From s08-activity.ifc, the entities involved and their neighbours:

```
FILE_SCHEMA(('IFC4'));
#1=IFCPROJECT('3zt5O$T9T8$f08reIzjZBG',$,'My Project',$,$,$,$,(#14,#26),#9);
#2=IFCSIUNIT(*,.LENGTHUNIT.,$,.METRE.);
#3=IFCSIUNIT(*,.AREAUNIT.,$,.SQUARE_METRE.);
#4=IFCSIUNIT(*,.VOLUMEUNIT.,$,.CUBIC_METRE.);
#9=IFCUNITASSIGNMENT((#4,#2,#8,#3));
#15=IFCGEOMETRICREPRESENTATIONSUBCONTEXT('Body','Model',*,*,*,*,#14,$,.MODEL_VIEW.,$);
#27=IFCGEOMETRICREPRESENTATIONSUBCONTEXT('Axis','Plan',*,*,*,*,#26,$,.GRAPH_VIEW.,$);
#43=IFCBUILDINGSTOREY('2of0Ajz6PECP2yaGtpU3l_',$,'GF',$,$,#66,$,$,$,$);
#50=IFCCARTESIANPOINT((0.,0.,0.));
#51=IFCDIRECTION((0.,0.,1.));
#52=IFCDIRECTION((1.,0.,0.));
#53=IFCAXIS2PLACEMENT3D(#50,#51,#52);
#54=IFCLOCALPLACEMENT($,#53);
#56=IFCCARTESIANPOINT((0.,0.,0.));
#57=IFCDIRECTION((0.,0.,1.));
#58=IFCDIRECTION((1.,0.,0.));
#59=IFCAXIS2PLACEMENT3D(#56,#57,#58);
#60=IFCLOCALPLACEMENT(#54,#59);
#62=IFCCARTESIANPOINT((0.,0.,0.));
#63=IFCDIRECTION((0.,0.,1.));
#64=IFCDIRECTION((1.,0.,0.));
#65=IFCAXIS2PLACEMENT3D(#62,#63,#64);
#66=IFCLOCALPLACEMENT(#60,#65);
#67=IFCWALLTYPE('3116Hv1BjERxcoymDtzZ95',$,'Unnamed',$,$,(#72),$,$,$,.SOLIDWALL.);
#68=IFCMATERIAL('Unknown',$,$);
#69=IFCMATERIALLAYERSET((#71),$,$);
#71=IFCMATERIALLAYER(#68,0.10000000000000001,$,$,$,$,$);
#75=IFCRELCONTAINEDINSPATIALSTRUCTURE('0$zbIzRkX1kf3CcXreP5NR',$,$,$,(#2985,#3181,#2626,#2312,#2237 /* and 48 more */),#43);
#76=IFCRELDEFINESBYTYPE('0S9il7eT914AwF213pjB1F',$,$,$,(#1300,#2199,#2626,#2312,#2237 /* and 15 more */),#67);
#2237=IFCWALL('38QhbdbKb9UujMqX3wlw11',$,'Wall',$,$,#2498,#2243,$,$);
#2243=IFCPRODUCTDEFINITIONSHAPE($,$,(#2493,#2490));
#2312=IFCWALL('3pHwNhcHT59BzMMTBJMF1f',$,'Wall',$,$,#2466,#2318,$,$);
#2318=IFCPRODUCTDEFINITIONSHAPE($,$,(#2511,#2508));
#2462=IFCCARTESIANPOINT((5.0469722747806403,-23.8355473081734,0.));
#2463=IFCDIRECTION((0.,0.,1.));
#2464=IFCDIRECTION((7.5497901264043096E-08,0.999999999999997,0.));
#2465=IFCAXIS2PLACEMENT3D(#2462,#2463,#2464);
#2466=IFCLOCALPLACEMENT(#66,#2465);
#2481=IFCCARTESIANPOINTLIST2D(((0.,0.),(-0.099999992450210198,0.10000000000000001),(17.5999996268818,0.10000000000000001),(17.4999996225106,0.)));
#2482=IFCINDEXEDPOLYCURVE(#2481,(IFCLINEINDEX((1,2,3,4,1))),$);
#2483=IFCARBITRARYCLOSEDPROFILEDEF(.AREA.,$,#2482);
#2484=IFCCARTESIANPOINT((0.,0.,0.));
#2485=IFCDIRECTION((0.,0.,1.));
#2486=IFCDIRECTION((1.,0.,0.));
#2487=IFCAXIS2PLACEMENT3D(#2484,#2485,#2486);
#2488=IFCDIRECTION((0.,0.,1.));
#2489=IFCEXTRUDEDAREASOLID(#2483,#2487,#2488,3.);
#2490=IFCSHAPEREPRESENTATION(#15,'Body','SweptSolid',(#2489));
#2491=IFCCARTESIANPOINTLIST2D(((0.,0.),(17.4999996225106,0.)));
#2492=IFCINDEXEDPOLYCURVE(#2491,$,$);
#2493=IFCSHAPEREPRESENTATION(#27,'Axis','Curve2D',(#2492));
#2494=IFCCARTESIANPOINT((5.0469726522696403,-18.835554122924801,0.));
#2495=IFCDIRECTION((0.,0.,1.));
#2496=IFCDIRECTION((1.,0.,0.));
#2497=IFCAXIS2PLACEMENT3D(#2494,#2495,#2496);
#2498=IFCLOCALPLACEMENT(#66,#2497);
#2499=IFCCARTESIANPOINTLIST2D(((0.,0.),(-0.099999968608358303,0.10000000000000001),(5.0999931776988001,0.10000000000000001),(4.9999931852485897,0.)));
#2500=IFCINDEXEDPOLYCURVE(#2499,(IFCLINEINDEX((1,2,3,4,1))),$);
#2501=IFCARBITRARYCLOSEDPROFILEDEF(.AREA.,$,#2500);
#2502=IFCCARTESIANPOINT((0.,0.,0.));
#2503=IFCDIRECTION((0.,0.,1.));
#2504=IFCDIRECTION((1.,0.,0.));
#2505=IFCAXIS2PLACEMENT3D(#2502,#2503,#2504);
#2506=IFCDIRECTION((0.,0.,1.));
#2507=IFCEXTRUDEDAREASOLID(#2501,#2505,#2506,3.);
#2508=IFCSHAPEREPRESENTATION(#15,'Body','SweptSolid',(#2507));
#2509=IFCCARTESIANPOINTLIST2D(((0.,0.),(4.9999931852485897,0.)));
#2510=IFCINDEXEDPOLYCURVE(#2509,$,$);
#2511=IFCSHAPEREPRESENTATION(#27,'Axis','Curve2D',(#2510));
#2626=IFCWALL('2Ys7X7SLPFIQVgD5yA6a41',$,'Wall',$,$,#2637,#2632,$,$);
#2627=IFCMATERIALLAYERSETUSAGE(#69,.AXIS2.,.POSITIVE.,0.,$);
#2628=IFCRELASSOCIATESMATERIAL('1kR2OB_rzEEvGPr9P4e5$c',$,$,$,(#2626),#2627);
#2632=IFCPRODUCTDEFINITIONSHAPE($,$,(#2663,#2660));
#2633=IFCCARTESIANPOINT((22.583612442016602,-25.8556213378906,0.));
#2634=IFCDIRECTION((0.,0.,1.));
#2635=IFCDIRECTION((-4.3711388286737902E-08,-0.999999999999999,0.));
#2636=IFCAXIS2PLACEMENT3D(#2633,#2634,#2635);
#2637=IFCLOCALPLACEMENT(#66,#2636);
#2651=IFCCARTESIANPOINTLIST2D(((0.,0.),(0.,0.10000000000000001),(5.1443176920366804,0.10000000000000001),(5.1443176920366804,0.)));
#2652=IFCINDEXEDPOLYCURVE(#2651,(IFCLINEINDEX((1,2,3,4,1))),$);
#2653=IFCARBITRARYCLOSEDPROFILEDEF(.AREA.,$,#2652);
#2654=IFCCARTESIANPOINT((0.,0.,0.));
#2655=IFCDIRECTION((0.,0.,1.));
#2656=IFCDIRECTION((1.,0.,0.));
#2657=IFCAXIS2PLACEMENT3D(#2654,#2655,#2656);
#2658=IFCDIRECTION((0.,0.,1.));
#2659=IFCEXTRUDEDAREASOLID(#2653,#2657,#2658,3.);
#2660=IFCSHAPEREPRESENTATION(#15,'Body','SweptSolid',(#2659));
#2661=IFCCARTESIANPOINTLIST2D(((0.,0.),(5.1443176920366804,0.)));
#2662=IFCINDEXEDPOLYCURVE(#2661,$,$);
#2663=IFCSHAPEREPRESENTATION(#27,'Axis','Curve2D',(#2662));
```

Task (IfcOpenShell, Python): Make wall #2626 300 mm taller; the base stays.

```python
import ifcopenshell
import ifcopenshell.geom
import ifcopenshell.util.representation
import ifcopenshell.util.shape

model = ifcopenshell.open("s08-activity.ifc")
settings = ifcopenshell.geom.settings()


def volume(element):
    """Net volume in cubic metres, openings subtracted."""
    shape = ifcopenshell.geom.create_shape(settings, element)
    return ifcopenshell.util.shape.get_volume(shape.geometry)


wall = model.by_guid("2Ys7X7SLPFIQVgD5yA6a41")
before = volume(wall)

body = ifcopenshell.util.representation.get_representation(wall, "Model", "Body")
solid = body.Items[0]
old_height = solid.Depth
solid.Depth += 0.3
after = volume(wall)

print(f"height {old_height:g} -> {solid.Depth:g}, volume {before:.3f} -> {after:.3f} m3")

model.write("s08-activity_edited.ifc")
```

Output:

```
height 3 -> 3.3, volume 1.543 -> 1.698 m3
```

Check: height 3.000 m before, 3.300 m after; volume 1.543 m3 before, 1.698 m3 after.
